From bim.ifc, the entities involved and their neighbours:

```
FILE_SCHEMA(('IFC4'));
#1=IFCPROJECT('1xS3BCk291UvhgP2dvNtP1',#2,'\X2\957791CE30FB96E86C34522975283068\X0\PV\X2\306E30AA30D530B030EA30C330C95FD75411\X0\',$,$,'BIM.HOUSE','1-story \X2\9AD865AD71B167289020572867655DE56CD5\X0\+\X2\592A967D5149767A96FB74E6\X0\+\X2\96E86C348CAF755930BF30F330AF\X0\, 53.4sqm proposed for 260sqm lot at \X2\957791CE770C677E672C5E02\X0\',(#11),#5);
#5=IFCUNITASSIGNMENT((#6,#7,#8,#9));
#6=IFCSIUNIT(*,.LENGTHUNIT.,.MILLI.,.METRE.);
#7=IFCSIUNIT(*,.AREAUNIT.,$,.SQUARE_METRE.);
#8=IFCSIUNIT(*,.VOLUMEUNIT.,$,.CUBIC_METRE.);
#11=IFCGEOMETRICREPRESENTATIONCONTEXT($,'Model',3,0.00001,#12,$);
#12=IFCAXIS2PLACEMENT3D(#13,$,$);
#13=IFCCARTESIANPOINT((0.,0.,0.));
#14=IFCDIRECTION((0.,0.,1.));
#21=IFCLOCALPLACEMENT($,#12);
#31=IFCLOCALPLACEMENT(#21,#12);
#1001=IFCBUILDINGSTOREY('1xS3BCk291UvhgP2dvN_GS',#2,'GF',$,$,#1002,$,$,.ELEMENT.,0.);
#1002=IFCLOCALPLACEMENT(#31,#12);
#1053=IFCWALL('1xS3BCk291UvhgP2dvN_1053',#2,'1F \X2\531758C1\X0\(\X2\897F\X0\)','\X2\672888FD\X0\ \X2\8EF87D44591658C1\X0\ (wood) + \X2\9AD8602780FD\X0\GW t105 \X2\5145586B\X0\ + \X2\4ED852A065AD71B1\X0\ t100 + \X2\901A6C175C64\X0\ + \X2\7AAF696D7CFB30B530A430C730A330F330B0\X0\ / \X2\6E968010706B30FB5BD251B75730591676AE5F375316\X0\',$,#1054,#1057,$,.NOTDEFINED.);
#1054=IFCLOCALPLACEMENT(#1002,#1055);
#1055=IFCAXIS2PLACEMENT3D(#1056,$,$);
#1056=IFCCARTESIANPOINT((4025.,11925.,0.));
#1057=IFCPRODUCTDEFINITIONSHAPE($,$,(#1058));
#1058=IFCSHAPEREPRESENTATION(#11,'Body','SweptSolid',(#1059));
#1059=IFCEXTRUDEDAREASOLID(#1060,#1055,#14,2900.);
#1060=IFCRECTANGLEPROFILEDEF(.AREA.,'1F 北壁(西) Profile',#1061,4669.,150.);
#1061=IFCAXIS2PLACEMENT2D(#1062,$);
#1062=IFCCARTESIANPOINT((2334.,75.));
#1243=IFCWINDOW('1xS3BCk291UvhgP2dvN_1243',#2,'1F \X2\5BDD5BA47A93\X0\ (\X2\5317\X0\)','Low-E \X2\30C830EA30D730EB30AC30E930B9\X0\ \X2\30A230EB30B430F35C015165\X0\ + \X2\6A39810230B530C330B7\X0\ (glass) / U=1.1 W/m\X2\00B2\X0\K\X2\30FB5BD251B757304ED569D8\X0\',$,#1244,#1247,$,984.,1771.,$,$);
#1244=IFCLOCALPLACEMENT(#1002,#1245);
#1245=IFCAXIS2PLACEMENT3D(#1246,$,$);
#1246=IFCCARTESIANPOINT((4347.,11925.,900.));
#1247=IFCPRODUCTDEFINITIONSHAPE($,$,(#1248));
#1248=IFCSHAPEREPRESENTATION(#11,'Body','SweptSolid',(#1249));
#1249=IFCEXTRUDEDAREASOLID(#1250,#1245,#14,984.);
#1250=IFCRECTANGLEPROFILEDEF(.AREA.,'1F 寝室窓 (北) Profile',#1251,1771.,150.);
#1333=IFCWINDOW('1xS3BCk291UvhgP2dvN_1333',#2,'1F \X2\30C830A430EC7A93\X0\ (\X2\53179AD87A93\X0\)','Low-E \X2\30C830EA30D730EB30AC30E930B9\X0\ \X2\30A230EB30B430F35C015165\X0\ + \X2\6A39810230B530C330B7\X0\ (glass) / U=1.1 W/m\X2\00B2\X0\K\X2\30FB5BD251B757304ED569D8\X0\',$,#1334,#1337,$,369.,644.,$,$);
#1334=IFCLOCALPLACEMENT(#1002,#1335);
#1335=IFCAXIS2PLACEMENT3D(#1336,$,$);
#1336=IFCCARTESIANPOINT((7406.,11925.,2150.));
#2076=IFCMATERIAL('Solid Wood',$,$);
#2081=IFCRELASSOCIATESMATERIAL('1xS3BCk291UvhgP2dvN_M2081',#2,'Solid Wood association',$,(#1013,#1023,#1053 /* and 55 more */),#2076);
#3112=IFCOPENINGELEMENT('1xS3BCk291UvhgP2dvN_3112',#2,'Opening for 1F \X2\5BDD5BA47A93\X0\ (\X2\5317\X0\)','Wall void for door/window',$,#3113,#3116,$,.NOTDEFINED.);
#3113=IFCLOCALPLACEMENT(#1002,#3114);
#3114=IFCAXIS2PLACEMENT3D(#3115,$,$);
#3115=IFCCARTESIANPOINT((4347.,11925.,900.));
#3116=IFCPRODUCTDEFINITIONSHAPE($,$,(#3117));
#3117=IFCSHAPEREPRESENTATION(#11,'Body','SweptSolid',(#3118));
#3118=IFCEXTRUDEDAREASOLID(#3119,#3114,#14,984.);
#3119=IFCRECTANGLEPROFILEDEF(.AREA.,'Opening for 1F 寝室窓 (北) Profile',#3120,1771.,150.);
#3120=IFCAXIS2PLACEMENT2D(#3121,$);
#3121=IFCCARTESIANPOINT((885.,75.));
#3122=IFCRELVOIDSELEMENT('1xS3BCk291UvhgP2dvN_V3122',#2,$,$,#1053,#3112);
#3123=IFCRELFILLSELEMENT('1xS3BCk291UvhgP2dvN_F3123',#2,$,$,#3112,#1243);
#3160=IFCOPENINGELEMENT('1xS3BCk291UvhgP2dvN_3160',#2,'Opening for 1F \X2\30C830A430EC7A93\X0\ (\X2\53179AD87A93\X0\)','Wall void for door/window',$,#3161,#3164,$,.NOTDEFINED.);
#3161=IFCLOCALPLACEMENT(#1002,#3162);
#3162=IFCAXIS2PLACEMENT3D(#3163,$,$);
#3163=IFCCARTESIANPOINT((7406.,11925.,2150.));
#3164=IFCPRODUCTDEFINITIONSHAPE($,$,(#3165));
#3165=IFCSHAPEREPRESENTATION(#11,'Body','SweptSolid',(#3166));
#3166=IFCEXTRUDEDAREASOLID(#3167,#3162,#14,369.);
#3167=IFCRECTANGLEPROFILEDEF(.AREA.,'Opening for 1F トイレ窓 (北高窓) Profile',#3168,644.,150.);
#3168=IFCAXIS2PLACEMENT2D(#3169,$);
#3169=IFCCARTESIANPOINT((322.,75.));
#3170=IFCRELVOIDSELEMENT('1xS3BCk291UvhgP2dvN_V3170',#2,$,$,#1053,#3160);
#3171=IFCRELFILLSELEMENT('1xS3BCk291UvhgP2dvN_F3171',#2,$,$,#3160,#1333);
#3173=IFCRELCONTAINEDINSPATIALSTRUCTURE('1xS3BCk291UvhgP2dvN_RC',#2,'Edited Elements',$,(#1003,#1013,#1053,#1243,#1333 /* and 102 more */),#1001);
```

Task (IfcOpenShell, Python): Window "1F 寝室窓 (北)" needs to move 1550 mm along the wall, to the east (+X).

```python
import ifcopenshell
import ifcopenshell.api.geometry
import ifcopenshell.util.placement
import ifcopenshell.util.unit

model = ifcopenshell.open("bim.ifc")
unit_scale = ifcopenshell.util.unit.calculate_unit_scale(model)

window = model.by_guid("1xS3BCk291UvhgP2dvN_1243")
opening = window.FillsVoids[0].RelatingOpeningElement
wall = opening.VoidsElements[0].RelatingBuildingElement

wall_matrix = ifcopenshell.util.placement.get_local_placement(wall.ObjectPlacement)
shift = wall_matrix[:3, 0] * 1.55 / unit_scale
before = ifcopenshell.util.placement.get_local_placement(window.ObjectPlacement)[:3, 3].copy()

# The window is not placed relative to its opening, so move both.
for product in (opening, window):
    matrix = ifcopenshell.util.placement.get_local_placement(product.ObjectPlacement)
    matrix[:3, 3] += shift
    ifcopenshell.api.geometry.edit_object_placement(model, product=product, matrix=matrix, is_si=False)

after = ifcopenshell.util.placement.get_local_placement(window.ObjectPlacement)[:3, 3]
print("window moved by", (after - before).round(3) + 0.0)

model.write("bim_v2.ifc")
```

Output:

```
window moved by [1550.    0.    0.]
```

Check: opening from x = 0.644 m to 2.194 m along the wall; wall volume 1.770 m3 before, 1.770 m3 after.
